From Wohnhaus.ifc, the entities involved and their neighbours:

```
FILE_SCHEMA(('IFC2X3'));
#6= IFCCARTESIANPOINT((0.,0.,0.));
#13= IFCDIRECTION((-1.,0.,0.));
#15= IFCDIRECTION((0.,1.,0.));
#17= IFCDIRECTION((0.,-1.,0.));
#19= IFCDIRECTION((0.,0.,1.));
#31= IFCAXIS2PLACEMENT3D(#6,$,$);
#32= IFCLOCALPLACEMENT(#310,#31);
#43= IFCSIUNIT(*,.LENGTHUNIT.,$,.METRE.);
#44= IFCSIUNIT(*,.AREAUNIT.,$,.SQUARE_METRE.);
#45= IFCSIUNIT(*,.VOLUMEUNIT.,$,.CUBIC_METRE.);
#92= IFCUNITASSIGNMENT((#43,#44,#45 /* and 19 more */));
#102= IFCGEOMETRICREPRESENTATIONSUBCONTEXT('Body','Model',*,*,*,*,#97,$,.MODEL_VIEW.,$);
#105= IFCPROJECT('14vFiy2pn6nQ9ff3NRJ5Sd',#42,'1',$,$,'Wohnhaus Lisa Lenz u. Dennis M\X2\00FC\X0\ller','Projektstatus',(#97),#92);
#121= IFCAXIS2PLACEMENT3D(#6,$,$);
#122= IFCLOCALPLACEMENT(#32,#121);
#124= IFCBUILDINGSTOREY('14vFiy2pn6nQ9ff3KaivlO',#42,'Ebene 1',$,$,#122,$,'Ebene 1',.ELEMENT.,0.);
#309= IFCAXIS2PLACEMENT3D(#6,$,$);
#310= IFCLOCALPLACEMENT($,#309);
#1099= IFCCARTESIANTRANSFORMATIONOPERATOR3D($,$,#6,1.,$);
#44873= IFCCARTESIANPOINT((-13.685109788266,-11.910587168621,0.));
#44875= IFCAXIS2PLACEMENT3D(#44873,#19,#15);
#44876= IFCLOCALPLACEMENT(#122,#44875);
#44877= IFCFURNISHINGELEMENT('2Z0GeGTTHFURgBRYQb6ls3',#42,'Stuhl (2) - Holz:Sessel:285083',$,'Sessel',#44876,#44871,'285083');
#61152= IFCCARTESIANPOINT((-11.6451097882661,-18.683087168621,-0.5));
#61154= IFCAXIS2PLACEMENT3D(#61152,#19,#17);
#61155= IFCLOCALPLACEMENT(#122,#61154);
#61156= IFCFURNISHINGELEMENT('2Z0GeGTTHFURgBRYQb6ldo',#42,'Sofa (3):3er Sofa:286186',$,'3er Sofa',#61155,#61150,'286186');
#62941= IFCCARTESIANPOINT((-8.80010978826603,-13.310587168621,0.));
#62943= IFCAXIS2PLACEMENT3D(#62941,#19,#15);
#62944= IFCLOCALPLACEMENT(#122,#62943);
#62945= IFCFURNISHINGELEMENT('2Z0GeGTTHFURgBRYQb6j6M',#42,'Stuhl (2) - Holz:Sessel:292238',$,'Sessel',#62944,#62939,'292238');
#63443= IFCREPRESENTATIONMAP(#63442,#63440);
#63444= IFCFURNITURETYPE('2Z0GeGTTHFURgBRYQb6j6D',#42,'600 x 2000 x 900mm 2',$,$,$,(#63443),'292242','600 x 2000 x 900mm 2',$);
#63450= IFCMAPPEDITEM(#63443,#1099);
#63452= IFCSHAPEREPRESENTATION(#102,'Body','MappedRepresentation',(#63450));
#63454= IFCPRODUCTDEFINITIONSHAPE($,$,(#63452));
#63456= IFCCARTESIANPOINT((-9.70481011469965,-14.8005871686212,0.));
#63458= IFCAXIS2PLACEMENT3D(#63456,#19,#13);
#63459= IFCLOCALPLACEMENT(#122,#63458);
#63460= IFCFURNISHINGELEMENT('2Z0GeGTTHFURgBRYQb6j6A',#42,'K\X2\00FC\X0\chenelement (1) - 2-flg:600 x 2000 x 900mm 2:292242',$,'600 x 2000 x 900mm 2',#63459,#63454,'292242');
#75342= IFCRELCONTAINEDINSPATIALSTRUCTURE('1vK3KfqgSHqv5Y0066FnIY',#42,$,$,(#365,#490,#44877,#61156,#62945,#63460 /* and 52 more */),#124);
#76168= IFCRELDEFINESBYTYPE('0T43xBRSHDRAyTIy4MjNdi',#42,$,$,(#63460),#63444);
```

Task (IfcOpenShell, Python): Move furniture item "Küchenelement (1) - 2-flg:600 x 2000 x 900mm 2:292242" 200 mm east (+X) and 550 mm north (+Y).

```python
import ifcopenshell
import ifcopenshell.api.geometry
import ifcopenshell.util.placement
import ifcopenshell.util.unit

model = ifcopenshell.open("Wohnhaus.ifc")
unit_scale = ifcopenshell.util.unit.calculate_unit_scale(model)

item = model.by_guid("2Z0GeGTTHFURgBRYQb6j6A")
matrix = ifcopenshell.util.placement.get_local_placement(item.ObjectPlacement)
matrix[0, 3] += 0.2 / unit_scale
matrix[1, 3] += 0.55 / unit_scale
ifcopenshell.api.geometry.edit_object_placement(model, product=item, matrix=matrix, is_si=False)

print(ifcopenshell.util.placement.get_local_placement(item.ObjectPlacement).round(3) + 0.0)

model.write("Wohnhaus_updated.ifc")
```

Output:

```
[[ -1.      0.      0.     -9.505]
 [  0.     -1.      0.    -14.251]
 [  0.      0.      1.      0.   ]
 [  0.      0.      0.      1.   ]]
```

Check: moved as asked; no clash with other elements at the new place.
